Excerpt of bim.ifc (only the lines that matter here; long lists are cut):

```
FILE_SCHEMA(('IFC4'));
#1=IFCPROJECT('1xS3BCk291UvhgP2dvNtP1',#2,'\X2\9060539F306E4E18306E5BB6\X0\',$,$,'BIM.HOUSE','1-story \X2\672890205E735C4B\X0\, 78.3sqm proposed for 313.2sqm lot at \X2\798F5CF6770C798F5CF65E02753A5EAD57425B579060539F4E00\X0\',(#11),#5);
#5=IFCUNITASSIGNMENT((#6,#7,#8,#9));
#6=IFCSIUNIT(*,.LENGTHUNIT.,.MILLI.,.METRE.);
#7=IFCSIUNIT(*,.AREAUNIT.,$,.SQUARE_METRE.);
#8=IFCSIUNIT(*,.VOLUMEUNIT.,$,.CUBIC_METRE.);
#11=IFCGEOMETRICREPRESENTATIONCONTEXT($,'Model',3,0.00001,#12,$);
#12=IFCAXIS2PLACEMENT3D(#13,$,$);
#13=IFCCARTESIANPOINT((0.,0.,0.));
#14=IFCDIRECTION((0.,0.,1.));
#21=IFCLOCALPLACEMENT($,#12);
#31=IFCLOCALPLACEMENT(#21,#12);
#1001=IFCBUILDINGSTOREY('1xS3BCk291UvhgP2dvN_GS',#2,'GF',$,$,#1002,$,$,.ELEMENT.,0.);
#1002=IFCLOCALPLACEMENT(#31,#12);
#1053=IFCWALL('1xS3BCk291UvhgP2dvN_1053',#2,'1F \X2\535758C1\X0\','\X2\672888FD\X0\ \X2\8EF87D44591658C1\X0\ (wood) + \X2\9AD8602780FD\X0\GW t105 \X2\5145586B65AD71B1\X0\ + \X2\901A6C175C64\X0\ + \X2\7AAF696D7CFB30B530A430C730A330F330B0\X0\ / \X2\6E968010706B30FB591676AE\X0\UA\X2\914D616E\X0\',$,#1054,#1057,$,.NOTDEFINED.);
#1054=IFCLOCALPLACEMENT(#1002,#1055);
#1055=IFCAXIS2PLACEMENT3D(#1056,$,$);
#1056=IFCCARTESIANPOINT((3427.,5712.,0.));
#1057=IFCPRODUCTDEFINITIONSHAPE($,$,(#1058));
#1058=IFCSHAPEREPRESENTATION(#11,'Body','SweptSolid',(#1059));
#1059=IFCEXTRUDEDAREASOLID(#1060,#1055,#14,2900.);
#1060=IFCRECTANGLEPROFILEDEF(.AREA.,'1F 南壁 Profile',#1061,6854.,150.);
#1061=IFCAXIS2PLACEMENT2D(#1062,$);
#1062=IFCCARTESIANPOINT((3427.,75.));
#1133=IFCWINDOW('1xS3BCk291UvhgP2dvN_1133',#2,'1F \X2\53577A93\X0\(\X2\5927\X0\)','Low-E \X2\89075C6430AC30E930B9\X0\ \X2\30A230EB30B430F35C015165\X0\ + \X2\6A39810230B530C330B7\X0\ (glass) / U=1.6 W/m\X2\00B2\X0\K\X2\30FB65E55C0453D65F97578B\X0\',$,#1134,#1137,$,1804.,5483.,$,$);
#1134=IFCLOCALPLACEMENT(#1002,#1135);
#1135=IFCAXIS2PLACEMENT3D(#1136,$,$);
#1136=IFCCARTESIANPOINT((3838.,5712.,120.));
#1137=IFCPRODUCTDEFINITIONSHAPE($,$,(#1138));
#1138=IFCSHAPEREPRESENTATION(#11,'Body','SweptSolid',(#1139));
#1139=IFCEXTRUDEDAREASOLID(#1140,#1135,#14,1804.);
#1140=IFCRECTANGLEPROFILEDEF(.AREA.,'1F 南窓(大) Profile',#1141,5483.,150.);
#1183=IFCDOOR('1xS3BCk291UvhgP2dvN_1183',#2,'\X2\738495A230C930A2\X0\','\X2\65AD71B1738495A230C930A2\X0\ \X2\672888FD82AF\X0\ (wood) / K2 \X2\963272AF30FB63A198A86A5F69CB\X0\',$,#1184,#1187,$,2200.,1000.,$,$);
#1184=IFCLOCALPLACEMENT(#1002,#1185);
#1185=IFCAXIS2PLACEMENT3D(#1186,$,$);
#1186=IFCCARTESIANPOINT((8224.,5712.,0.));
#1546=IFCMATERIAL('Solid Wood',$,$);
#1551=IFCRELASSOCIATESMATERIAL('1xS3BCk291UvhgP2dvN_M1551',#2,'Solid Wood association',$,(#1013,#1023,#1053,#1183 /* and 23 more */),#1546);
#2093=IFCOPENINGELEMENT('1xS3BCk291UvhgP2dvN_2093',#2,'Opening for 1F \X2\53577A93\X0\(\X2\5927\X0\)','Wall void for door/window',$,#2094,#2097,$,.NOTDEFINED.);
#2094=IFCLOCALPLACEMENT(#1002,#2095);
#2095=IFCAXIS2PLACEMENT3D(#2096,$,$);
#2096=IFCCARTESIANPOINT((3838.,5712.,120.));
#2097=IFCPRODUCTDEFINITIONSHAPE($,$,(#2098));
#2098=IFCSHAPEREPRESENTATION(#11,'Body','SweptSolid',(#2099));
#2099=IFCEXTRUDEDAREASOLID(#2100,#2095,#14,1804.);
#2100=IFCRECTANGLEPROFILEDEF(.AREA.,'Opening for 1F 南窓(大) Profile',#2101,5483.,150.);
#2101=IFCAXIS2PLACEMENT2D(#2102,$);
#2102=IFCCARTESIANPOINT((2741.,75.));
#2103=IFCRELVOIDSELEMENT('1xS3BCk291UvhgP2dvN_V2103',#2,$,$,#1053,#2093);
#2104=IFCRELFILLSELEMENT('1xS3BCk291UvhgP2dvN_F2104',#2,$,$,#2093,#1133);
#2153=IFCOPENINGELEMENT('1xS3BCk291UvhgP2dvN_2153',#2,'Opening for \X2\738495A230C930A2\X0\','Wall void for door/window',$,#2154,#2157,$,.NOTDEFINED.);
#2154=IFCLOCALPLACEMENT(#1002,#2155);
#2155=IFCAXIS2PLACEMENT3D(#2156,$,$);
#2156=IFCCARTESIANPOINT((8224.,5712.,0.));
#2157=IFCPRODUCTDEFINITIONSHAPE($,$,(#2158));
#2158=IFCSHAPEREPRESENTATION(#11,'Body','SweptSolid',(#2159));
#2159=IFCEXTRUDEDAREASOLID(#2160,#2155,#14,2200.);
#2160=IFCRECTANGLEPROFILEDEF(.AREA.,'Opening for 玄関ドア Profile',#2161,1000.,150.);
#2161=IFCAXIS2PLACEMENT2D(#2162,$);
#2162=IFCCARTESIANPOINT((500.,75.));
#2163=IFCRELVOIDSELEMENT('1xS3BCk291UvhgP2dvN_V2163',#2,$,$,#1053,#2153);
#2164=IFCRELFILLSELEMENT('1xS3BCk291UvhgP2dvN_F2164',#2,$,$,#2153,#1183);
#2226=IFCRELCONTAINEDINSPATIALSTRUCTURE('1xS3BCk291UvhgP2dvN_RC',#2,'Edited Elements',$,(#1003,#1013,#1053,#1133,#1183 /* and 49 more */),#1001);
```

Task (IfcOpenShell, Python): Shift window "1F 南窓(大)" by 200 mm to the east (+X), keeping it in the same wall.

```python
import ifcopenshell
import ifcopenshell.api.geometry
import ifcopenshell.util.placement

model = ifcopenshell.open("bim.ifc")

window = model.by_guid("1xS3BCk291UvhgP2dvN_1133")
opening = window.FillsVoids[0].RelatingOpeningElement
wall = opening.VoidsElements[0].RelatingBuildingElement

wall_matrix = ifcopenshell.util.placement.get_local_placement(wall.ObjectPlacement)
shift = wall_matrix[:3, 0] * 200.0
before = ifcopenshell.util.placement.get_local_placement(window.ObjectPlacement)[:3, 3].copy()

# The window is not placed relative to its opening, so move both.
for product in (opening, window):
    matrix = ifcopenshell.util.placement.get_local_placement(product.ObjectPlacement)
    matrix[:3, 3] += shift
    ifcopenshell.api.geometry.edit_object_placement(model, product=product, matrix=matrix, is_si=False)

after = ifcopenshell.util.placement.get_local_placement(window.ObjectPlacement)[:3, 3]
print("window moved by", (after - before).round(3) + 0.0)

model.write("bim_updated.ifc")
```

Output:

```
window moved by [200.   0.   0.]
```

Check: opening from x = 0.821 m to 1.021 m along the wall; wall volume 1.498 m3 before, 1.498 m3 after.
